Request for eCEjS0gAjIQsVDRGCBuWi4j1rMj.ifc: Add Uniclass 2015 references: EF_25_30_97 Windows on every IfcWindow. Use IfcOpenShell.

First a look at what the model holds.

```python
import ifcopenshell

model = ifcopenshell.open("eCEjS0gAjIQsVDRGCBuWi4j1rMj.ifc")
print(model.schema)
print("classifications:", [c.Name for c in model.by_type("IfcClassification")])
for ifc_class in ("IfcDoor", "IfcRoof", "IfcStair", "IfcWall", "IfcWindow"):
    print(ifc_class, len(model.by_type(ifc_class)))
```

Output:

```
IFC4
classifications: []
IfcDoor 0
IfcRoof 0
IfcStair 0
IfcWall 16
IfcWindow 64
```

```python
import ifcopenshell
import ifcopenshell.api.classification

model = ifcopenshell.open("eCEjS0gAjIQsVDRGCBuWi4j1rMj.ifc")

system = ifcopenshell.api.classification.add_classification(model, classification="Uniclass 2015")

codes = {
    "IfcWindow": ("EF_25_30_97", "Windows"),
}
for ifc_class, (code, name) in codes.items():
    products = model.by_type(ifc_class)
    ifcopenshell.api.classification.add_reference(
        model, products=products, classification=system, identification=code, name=name
    )
    print(code, len(products))

model.write("eCEjS0gAjIQsVDRGCBuWi4j1rMj_edited.ifc")
```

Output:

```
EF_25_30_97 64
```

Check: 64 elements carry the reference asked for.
